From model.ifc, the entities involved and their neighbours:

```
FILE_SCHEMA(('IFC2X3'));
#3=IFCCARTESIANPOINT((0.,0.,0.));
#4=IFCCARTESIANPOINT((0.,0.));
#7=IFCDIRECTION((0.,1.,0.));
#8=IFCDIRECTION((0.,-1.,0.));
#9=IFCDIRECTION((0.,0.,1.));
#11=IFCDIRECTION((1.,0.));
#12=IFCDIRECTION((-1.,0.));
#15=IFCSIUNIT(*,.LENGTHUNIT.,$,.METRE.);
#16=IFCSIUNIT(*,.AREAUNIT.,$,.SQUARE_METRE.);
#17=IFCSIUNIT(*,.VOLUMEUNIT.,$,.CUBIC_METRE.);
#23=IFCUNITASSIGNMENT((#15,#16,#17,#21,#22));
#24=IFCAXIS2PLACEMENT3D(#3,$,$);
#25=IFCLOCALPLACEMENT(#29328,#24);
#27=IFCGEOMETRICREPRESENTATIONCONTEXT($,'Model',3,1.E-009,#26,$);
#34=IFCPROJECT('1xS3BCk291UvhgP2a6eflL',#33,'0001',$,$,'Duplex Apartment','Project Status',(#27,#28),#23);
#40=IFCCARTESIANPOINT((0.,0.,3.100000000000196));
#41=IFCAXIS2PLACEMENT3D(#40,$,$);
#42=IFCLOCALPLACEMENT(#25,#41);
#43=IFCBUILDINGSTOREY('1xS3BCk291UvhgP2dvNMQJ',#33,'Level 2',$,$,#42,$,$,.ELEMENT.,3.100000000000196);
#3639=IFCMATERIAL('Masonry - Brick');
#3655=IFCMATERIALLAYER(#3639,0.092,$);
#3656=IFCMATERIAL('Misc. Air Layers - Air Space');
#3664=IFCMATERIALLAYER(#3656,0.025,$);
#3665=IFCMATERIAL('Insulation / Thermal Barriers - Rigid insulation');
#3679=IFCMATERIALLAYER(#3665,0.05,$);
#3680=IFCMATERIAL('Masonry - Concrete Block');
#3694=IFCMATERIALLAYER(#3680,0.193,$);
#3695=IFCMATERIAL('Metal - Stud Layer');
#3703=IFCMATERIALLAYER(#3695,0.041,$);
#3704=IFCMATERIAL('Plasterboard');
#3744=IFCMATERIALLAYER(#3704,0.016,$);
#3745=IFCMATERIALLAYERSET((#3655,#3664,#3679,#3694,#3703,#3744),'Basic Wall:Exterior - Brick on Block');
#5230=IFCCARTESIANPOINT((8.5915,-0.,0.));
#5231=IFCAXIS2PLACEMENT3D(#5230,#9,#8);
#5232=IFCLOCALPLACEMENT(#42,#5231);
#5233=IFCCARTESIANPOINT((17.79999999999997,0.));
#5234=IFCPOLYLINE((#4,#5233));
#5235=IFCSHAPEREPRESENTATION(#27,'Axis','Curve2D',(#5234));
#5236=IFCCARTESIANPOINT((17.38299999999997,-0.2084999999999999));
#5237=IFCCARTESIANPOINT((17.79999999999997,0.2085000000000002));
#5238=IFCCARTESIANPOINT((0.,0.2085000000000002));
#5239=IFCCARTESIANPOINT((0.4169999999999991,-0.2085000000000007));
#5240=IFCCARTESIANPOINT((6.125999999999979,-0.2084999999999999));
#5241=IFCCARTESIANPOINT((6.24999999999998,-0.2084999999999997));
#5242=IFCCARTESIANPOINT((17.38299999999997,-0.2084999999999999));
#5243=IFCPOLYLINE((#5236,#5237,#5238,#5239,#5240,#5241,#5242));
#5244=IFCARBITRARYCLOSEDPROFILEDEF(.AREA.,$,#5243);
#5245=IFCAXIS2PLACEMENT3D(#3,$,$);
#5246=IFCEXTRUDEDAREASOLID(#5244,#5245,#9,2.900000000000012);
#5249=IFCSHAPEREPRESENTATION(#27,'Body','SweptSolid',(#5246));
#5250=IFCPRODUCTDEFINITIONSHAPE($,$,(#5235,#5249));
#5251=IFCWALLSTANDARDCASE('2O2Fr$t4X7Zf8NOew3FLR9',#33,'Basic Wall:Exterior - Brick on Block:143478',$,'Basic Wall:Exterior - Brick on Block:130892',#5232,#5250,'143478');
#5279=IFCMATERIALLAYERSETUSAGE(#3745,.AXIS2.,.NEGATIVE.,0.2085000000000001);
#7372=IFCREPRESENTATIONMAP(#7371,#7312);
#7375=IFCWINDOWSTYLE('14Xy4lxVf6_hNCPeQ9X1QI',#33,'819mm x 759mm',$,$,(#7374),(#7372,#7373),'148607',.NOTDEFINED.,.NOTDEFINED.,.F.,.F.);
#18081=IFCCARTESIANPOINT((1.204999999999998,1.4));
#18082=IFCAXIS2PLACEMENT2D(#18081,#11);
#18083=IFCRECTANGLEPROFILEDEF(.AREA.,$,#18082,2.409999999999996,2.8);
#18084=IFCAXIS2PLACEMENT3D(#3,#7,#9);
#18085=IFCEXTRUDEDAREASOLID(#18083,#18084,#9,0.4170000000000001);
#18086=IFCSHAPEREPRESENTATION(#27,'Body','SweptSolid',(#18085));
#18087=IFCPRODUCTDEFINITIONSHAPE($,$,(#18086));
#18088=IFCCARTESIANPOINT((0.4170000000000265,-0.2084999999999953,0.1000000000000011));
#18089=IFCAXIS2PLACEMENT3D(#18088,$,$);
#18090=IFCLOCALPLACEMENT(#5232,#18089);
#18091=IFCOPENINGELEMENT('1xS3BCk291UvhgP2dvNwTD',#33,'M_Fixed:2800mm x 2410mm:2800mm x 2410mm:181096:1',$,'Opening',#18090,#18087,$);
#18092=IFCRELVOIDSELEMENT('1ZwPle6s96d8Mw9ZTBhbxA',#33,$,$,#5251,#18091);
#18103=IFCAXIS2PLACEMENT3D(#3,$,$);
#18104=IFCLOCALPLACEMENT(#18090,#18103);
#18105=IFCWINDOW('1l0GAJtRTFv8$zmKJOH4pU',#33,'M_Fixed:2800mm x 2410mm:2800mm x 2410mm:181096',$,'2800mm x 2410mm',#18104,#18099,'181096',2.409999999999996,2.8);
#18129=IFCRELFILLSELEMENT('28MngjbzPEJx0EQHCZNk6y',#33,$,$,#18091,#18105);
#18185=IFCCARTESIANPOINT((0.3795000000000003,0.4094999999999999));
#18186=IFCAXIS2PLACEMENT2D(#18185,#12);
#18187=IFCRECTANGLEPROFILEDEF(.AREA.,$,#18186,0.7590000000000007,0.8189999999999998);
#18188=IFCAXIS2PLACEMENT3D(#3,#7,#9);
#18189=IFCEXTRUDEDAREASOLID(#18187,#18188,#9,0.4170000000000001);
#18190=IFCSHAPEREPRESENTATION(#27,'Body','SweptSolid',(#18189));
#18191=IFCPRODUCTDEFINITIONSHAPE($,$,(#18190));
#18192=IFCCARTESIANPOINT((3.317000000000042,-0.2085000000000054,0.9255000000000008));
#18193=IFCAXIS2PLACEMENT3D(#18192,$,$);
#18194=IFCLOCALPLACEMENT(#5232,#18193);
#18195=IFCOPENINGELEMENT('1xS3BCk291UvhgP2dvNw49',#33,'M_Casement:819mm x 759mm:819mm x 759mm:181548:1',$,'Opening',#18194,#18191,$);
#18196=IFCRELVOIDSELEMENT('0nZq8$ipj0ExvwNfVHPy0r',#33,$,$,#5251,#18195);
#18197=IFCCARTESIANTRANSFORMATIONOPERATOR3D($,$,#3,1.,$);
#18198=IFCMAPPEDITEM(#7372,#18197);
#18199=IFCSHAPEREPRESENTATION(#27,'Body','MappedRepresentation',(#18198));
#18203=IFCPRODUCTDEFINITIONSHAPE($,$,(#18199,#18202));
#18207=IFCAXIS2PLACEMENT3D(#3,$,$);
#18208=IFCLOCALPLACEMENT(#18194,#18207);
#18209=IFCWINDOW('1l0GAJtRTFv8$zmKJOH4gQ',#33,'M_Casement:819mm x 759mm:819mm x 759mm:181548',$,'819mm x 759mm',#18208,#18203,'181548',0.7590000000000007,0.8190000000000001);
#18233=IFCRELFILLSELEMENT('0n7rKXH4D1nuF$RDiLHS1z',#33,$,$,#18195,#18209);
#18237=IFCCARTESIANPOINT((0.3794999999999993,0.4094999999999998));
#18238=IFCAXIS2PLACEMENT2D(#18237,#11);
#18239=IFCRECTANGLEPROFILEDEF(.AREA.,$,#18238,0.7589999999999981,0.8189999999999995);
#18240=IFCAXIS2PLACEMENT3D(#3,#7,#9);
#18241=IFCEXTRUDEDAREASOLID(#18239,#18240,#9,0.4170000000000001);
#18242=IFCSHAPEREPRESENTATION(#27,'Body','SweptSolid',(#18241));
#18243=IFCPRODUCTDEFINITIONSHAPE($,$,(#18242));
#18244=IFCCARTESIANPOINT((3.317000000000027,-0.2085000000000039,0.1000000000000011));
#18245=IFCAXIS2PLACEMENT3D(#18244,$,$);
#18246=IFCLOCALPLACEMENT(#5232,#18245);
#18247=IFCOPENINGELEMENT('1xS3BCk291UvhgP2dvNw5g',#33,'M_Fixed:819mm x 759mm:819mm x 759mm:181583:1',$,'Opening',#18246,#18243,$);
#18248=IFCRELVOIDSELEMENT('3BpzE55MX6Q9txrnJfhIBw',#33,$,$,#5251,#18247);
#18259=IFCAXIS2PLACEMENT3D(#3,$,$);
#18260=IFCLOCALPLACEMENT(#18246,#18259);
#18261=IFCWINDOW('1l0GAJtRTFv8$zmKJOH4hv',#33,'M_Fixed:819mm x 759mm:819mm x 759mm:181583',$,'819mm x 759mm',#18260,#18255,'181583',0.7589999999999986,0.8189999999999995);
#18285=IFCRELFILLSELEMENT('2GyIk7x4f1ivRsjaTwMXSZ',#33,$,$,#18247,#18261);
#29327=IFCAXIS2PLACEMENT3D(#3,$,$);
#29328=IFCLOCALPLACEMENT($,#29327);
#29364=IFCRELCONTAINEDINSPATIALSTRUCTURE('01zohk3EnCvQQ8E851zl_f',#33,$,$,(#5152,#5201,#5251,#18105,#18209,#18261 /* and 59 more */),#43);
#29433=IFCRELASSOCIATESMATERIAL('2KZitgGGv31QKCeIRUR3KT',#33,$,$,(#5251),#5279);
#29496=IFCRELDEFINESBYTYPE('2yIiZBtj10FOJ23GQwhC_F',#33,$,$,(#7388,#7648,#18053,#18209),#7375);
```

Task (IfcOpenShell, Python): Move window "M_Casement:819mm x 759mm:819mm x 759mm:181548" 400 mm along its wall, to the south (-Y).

```python
import ifcopenshell
import ifcopenshell.api.geometry
import ifcopenshell.util.placement
import ifcopenshell.util.unit

model = ifcopenshell.open("model.ifc")
unit_scale = ifcopenshell.util.unit.calculate_unit_scale(model)

window = model.by_guid("1l0GAJtRTFv8$zmKJOH4gQ")
opening = window.FillsVoids[0].RelatingOpeningElement
wall = opening.VoidsElements[0].RelatingBuildingElement

wall_matrix = ifcopenshell.util.placement.get_local_placement(wall.ObjectPlacement)
shift = wall_matrix[:3, 0] * 0.4 / unit_scale
before = ifcopenshell.util.placement.get_local_placement(window.ObjectPlacement)[:3, 3].copy()

# The window is placed relative to its opening, so it follows when the opening moves.
matrix = ifcopenshell.util.placement.get_local_placement(opening.ObjectPlacement)
matrix[:3, 3] += shift
ifcopenshell.api.geometry.edit_object_placement(
    model, product=opening, matrix=matrix, is_si=False, should_transform_children=True
)

after = ifcopenshell.util.placement.get_local_placement(window.ObjectPlacement)[:3, 3]
print("window moved by", (after - before).round(3) + 0.0)

model.write("model_edited.ifc")
```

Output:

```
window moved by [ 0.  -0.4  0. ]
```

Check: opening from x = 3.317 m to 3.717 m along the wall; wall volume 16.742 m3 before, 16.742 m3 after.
